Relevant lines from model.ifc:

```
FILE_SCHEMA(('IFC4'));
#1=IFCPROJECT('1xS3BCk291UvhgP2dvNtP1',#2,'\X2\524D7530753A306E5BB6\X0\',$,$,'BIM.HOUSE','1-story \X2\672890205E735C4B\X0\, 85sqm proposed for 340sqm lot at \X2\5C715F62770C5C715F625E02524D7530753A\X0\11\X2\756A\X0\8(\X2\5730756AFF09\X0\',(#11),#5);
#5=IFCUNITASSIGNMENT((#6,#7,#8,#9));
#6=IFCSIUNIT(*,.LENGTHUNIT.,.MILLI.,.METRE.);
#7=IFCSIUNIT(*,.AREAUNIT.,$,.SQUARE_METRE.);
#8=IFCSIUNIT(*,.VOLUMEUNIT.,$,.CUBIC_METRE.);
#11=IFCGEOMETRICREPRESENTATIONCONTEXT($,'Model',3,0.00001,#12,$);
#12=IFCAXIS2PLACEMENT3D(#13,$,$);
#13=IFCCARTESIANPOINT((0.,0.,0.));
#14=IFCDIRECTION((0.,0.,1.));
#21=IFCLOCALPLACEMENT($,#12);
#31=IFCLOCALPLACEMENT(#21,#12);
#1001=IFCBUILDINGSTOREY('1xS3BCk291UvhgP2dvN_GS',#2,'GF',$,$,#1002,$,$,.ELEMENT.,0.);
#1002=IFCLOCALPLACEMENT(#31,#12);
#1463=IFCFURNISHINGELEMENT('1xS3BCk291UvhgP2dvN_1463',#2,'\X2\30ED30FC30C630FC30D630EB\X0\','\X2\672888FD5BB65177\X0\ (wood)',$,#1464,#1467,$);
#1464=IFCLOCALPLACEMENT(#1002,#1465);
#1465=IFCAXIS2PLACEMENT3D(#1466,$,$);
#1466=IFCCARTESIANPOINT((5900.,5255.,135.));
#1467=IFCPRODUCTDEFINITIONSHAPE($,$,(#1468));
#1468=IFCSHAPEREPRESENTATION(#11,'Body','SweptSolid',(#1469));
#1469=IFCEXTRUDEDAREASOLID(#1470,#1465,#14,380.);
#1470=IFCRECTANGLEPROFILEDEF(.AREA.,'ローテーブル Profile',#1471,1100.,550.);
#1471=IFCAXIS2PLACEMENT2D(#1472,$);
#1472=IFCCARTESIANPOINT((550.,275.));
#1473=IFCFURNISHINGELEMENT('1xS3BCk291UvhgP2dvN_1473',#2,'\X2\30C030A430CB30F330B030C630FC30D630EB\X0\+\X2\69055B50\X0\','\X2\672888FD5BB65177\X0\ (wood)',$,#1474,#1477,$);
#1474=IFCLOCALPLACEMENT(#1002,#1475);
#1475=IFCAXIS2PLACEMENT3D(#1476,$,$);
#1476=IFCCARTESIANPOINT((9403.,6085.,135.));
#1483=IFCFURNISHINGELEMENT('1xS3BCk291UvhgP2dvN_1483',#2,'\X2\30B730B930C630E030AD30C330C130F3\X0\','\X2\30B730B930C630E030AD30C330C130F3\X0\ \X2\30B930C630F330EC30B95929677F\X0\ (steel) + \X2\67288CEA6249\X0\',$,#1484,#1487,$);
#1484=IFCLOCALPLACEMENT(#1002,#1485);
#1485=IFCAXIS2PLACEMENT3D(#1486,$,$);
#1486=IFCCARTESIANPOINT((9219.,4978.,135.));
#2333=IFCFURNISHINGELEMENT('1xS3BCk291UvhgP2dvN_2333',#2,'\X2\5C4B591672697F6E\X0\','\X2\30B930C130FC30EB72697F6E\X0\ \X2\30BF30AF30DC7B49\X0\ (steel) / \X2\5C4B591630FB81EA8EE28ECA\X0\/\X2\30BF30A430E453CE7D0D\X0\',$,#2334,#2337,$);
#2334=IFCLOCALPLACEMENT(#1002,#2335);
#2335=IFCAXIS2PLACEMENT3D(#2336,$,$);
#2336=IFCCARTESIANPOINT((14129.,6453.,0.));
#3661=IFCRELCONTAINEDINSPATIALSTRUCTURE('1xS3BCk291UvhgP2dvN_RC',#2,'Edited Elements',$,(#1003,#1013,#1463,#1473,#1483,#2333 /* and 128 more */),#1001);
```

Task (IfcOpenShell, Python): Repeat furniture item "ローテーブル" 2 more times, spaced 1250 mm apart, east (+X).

```python
import numpy as np
import ifcopenshell
import ifcopenshell.api.geometry
import ifcopenshell.api.root
import ifcopenshell.util.element
import ifcopenshell.util.placement
import ifcopenshell.util.unit

model = ifcopenshell.open("model.ifc")
unit_scale = ifcopenshell.util.unit.calculate_unit_scale(model)


def reuse_history(source, copy):
    """copy_class also copies each property set's owner history, people and application; keep the originals."""
    for rel in copy.IsDefinedBy:
        if rel.is_a("IfcRelDefinesByProperties") and (history := rel.RelatingPropertyDefinition.OwnerHistory):
            rel.RelatingPropertyDefinition.OwnerHistory = source.OwnerHistory
            ifcopenshell.util.element.remove_deep2(model, history)


source = model.by_guid("1xS3BCk291UvhgP2dvN_1463")
base = ifcopenshell.util.placement.get_local_placement(source.ObjectPlacement)
step = np.array([1.0, 0.0, 0.0]) * 1.25 / unit_scale

for i in range(1, 3):
    copy = ifcopenshell.api.root.copy_class(model, product=source)
    copy.Representation = ifcopenshell.util.element.copy_deep(
        model, source.Representation, exclude=["IfcGeometricRepresentationContext", "IfcRepresentationMap"]
    )
    reuse_history(source, copy)
    matrix = base.copy()
    matrix[:3, 3] += i * step
    print("added at", matrix[:3, 3].round(3) + 0.0)
    ifcopenshell.api.geometry.edit_object_placement(model, product=copy, matrix=matrix, is_si=False)

model.write("model_updated.ifc")
```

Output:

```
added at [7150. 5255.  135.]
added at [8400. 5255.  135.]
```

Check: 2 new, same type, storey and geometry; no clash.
